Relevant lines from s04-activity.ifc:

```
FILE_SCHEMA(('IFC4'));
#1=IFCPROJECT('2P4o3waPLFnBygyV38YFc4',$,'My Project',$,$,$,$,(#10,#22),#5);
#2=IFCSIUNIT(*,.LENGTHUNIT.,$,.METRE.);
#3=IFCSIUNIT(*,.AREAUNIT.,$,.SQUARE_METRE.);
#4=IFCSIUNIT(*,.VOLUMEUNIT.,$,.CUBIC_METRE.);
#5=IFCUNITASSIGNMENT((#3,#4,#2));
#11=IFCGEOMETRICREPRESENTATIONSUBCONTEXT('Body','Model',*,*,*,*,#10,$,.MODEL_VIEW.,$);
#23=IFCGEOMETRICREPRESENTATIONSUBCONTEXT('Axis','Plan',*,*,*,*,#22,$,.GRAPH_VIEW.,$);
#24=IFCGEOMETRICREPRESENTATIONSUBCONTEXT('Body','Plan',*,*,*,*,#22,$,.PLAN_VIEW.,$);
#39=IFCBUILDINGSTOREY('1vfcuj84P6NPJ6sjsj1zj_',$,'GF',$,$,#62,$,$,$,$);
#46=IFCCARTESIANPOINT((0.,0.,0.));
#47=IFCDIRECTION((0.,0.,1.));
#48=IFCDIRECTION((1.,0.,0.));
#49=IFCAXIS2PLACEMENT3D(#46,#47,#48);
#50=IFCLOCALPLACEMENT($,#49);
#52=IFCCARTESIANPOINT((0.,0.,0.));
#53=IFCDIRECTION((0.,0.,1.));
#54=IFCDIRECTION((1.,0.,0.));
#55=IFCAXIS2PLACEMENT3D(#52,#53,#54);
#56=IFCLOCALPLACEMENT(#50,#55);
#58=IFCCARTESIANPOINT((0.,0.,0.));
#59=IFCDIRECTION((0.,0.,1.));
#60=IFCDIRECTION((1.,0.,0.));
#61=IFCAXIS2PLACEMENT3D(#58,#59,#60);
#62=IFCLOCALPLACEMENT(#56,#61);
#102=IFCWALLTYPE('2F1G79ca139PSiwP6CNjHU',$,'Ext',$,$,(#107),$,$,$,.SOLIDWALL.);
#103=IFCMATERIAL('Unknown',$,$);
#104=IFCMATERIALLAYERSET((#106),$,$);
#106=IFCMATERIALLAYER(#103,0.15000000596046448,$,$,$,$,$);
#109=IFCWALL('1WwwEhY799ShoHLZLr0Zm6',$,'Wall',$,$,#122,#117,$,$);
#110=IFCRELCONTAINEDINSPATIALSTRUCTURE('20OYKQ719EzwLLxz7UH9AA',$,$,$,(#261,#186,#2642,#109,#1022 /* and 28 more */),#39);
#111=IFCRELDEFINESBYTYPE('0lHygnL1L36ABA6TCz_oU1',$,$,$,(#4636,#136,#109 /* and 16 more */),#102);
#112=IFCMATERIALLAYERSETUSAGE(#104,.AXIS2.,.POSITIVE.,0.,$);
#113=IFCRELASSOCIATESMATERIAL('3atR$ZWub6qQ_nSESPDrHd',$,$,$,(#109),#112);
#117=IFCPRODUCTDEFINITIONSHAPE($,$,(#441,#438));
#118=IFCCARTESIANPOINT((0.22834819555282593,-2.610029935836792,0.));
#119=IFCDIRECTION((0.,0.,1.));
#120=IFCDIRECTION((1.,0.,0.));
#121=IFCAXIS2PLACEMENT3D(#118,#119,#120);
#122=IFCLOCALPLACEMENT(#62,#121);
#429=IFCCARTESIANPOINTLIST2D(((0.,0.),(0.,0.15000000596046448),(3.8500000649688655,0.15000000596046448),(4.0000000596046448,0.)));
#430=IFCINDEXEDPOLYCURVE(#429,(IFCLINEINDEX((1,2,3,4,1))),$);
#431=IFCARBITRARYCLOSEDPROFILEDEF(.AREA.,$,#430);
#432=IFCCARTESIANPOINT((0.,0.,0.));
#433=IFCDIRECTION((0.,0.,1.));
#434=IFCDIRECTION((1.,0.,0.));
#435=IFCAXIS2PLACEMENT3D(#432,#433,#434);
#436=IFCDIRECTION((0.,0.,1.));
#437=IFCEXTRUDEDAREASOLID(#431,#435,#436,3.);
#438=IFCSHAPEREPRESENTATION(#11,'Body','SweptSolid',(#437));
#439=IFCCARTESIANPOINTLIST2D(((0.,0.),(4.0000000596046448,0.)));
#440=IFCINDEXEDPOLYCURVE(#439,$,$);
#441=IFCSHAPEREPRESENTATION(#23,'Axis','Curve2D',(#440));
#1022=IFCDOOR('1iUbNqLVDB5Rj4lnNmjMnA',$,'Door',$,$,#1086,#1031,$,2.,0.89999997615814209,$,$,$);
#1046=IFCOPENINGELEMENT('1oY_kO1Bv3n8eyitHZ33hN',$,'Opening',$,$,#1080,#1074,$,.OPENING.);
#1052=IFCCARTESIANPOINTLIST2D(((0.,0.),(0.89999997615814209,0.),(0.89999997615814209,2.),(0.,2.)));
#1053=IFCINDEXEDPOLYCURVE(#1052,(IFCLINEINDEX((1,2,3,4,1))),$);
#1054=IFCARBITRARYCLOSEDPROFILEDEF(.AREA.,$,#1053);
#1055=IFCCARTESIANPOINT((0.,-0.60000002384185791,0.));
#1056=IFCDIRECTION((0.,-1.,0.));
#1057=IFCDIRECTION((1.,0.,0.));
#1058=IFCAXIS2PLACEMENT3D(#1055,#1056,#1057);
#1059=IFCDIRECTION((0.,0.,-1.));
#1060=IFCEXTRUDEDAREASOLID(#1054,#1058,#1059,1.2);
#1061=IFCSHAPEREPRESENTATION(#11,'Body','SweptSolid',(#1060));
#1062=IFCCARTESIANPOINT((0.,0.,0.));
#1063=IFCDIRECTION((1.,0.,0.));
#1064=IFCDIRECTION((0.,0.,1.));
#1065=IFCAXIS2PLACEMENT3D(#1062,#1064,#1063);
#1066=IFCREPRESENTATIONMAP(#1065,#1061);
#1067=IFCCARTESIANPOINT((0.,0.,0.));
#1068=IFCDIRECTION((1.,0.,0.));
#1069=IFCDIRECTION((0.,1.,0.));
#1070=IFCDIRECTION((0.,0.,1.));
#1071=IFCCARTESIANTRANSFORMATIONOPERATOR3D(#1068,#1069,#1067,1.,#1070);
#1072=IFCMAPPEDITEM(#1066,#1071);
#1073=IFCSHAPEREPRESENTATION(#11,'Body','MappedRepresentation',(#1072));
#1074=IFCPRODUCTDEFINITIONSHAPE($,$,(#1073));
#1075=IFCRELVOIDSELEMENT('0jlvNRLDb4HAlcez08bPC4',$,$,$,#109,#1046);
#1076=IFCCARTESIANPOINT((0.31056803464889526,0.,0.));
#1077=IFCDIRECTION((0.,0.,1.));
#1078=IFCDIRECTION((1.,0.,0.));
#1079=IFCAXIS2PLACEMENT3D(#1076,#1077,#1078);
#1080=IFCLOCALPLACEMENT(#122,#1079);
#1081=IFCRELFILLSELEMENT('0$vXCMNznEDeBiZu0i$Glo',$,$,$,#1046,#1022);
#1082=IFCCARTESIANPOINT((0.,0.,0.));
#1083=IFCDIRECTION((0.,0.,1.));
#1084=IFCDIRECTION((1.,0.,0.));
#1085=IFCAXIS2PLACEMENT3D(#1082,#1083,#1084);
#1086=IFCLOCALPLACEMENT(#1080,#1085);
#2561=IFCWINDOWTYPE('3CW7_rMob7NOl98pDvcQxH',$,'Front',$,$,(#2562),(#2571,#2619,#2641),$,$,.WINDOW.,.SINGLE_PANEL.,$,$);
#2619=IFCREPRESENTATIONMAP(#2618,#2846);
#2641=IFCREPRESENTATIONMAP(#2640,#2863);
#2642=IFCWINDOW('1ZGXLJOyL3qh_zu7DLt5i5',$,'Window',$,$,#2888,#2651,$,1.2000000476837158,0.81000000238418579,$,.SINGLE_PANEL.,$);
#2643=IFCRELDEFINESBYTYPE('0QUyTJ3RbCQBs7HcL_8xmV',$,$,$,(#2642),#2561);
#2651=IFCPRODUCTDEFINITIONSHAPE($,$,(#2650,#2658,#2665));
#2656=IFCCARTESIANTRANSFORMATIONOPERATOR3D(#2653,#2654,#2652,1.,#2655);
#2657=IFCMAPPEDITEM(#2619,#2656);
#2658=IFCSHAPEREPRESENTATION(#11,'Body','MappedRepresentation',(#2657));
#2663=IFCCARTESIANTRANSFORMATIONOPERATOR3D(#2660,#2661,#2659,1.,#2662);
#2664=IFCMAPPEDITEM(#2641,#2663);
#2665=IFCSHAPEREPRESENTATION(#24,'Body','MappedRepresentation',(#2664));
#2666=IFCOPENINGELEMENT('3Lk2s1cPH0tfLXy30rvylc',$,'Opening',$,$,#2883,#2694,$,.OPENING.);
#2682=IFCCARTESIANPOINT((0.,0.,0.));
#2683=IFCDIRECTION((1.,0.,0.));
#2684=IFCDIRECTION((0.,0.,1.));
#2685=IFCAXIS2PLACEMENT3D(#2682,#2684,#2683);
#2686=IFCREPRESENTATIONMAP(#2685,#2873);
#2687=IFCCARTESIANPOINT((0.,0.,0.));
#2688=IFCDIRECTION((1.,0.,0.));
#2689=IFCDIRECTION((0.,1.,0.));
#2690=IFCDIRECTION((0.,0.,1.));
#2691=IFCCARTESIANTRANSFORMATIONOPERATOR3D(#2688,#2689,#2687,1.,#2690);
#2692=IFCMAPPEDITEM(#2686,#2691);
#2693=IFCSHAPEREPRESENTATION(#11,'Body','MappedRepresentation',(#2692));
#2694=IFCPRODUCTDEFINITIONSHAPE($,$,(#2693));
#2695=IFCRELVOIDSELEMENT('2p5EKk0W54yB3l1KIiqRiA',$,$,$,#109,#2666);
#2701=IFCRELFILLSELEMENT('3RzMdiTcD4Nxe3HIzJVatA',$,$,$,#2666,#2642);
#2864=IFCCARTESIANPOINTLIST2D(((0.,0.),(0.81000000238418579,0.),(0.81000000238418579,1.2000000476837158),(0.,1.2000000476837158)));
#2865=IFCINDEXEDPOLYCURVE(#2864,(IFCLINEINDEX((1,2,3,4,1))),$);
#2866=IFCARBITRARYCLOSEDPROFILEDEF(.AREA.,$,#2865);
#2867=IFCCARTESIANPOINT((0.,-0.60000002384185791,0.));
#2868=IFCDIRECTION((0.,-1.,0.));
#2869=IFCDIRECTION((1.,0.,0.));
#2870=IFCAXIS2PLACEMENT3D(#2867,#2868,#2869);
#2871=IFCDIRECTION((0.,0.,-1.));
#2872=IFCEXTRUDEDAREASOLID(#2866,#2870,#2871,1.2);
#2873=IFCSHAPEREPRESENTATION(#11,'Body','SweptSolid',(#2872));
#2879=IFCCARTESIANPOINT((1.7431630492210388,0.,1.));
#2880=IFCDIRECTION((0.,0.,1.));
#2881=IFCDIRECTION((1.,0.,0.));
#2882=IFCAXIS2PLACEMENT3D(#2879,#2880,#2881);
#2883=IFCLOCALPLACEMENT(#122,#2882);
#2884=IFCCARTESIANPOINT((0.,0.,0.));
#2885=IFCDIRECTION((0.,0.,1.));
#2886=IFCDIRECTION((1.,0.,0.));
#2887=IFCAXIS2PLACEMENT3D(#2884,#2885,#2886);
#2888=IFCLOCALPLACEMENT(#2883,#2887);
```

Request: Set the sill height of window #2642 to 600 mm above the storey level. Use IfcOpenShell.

```python
import numpy as np
import ifcopenshell
import ifcopenshell.api.geometry
import ifcopenshell.geom
import ifcopenshell.util.element
import ifcopenshell.util.placement
import ifcopenshell.util.shape
import ifcopenshell.util.unit

model = ifcopenshell.open("s04-activity.ifc")
unit_scale = ifcopenshell.util.unit.calculate_unit_scale(model)

window = model.by_guid("1ZGXLJOyL3qh_zu7DLt5i5")
opening = window.FillsVoids[0].RelatingOpeningElement
storey = ifcopenshell.util.element.get_container(window, ifc_class="IfcBuildingStorey")
level = ifcopenshell.util.placement.get_local_placement(storey.ObjectPlacement)[2, 3]

# The opening's origin need not be at the sill, so measure its lowest point.
shape = ifcopenshell.geom.create_shape(ifcopenshell.geom.settings(), opening)
bottom = ifcopenshell.util.shape.get_shape_bottom_elevation(shape, shape.geometry) / unit_scale
dz = level + 0.6 / unit_scale - bottom

shift = np.array([0.0, 0.0, dz])
# The window is placed relative to its opening, so it follows when the opening moves.
matrix = ifcopenshell.util.placement.get_local_placement(opening.ObjectPlacement)
matrix[:3, 3] += shift
ifcopenshell.api.geometry.edit_object_placement(
    model, product=opening, matrix=matrix, is_si=False, should_transform_children=True
)

print(f"moved by {dz * unit_scale:+.3f} m")

model.write("s04-activity_v2.ifc")
```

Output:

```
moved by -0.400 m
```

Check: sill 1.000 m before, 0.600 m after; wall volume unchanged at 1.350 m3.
